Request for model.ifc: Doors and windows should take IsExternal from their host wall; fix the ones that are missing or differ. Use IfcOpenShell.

First a look at what the model holds.

```python
import ifcopenshell
import ifcopenshell.util.element

model = ifcopenshell.open("model.ifc")
print(model.schema)
seen = {}
for e in model.by_type("IfcDoor") + model.by_type("IfcWindow"):
    if not e.FillsVoids:
        continue
    host = e.FillsVoids[0].RelatingOpeningElement.VoidsElements[0].RelatingBuildingElement
    own = ifcopenshell.util.element.get_pset(e, f"Pset_{e.is_a()[3:].removesuffix('StandardCase')}Common", "IsExternal")
    wall = ifcopenshell.util.element.get_pset(host, "Pset_WallCommon", "IsExternal")
    seen[e.is_a(), own, wall] = seen.get((e.is_a(), own, wall), 0) + 1
for (cls, own, wall), count in sorted(seen.items(), key=str):
    print(count, cls, "IsExternal:", own, "| host wall:", wall)
```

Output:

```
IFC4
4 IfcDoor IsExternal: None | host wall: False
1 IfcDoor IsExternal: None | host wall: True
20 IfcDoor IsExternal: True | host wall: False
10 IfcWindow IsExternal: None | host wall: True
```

```python
import ifcopenshell
import ifcopenshell.api.pset
import ifcopenshell.util.element

model = ifcopenshell.open("model.ifc")

count = 0
for ifc_class, pset_name in (("IfcDoor", "Pset_DoorCommon"), ("IfcWindow", "Pset_WindowCommon")):
    for e in model.by_type(ifc_class):
        if not e.FillsVoids:
            continue
        host = e.FillsVoids[0].RelatingOpeningElement.VoidsElements[0].RelatingBuildingElement
        external = ifcopenshell.util.element.get_pset(host, "Pset_WallCommon", "IsExternal")
        if external is None or ifcopenshell.util.element.get_pset(e, pset_name, "IsExternal") == external:
            continue
        pset = ifcopenshell.api.pset.add_pset(model, product=e, name=pset_name)
        ifcopenshell.api.pset.edit_pset(model, pset=pset, properties={"IsExternal": external})
        count += 1

print(count, "updated")

model.write("model_rev.ifc")
```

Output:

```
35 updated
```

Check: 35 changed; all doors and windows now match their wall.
